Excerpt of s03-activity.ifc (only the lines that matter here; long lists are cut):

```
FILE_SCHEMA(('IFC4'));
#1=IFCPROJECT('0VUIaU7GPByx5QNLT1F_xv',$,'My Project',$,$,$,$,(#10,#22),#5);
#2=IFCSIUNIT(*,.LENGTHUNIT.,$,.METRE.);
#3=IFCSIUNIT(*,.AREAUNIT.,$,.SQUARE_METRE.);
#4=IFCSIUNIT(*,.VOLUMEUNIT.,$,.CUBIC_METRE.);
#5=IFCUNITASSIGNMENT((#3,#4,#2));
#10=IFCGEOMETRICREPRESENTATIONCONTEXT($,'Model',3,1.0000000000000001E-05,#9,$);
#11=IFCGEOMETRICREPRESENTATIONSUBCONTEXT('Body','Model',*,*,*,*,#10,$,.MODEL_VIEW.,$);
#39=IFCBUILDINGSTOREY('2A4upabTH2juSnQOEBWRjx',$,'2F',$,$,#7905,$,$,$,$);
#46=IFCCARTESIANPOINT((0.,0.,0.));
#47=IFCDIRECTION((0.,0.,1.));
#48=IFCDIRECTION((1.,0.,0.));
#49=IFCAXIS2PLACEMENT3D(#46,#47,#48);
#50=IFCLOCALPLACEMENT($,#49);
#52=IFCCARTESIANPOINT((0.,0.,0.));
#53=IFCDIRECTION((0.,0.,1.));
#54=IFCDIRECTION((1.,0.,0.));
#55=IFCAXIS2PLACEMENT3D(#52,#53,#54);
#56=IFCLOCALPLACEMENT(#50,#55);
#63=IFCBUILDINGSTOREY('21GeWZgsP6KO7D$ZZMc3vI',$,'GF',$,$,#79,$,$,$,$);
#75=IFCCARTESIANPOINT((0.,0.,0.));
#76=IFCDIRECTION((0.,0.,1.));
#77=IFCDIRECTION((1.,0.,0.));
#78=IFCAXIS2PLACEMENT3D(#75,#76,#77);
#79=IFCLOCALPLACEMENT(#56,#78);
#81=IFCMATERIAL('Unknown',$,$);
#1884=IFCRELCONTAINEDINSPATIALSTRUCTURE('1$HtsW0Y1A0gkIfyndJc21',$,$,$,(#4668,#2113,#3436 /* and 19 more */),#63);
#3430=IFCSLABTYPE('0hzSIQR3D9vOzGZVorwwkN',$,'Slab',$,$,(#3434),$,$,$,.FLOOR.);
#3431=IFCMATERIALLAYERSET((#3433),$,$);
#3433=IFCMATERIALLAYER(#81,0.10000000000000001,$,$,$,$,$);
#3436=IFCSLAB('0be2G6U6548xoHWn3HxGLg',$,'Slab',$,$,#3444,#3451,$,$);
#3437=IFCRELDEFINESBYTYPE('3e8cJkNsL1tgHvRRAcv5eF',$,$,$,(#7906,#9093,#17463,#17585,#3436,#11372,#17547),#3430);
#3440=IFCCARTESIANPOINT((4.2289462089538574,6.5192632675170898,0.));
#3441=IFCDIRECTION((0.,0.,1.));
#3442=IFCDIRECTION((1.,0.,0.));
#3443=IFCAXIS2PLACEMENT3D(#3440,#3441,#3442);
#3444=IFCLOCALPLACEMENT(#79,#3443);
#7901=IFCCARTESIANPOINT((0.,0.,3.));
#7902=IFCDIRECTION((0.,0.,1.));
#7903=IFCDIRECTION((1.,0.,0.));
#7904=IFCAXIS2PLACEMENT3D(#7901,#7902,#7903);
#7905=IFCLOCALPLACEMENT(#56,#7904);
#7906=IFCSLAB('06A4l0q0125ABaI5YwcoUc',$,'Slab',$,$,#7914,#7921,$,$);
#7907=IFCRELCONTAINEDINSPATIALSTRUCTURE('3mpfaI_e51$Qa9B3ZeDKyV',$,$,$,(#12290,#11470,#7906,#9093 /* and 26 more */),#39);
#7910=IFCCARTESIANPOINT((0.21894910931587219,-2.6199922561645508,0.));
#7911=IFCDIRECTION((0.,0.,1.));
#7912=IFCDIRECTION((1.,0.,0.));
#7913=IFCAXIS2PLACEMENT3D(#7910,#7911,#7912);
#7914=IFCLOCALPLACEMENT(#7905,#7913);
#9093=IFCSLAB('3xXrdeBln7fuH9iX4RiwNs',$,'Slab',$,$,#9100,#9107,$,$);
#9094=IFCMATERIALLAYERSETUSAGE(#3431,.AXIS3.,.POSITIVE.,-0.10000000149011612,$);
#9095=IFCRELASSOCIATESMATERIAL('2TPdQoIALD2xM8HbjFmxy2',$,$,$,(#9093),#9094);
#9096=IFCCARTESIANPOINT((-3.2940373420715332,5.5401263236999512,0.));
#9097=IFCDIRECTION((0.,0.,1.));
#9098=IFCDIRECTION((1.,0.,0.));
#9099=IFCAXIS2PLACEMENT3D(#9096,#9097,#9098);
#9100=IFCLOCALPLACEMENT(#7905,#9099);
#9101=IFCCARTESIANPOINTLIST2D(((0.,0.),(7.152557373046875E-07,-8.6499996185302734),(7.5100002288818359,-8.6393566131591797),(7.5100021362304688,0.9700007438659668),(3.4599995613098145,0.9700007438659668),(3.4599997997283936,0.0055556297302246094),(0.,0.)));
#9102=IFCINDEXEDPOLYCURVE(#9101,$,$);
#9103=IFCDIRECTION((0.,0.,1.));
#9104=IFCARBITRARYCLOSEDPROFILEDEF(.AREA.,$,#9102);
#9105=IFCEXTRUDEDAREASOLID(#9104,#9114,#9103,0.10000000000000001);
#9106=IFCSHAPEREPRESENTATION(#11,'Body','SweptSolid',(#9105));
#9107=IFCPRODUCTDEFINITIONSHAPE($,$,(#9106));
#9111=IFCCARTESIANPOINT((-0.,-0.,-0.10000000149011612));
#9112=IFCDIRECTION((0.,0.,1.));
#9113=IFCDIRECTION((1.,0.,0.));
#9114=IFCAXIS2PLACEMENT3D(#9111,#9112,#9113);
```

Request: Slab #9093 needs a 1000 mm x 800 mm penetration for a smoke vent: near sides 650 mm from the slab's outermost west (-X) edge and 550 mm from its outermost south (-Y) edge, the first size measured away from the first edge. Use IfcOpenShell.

```python
import numpy as np
import ifcopenshell
import ifcopenshell.api.feature
import ifcopenshell.api.geometry
import ifcopenshell.api.root
import ifcopenshell.geom
import ifcopenshell.util.placement
import ifcopenshell.util.representation
import ifcopenshell.util.shape
import ifcopenshell.util.unit

model = ifcopenshell.open("s03-activity.ifc")
unit_scale = ifcopenshell.util.unit.calculate_unit_scale(model)
settings = ifcopenshell.geom.settings()


def volume(element):
    """Net volume in cubic metres, openings subtracted."""
    shape = ifcopenshell.geom.create_shape(settings, element)
    return ifcopenshell.util.shape.get_volume(shape.geometry)


slab = model.by_guid("3xXrdeBln7fuH9iX4RiwNs")
before = volume(slab)

# Extent in the slab's own axes, in metres. The edges named are its -X and -Y sides.
slab_shape = ifcopenshell.geom.create_shape(settings, slab)
vertices = ifcopenshell.util.shape.get_vertices(slab_shape.geometry)
x_min, y_min, bottom = vertices.min(axis=0)
top = vertices[:, 2].max()

opening = ifcopenshell.api.root.create_entity(model, ifc_class="IfcOpeningElement", name="Smoke vent opening", predefined_type="OPENING")
context = ifcopenshell.util.representation.get_context(model, "Model", "Body", "MODEL_VIEW")
width, depth = 1, 0.8
outline = [(0.0, 0.0), (width, 0.0), (width, depth), (0.0, depth), (0.0, 0.0)]
# Overshoot both faces by 50 mm so the cut is clean.
shape = ifcopenshell.api.geometry.add_slab_representation(
    model, context=context, depth=top - bottom + 0.1, polyline=outline
)
ifcopenshell.api.geometry.assign_representation(model, product=opening, representation=shape)

matrix = ifcopenshell.util.placement.get_local_placement(slab.ObjectPlacement)
matrix[:, 3] = matrix @ np.append(np.array([x_min + 0.65, y_min + 0.55, bottom - 0.05]) / unit_scale, 1.0)
ifcopenshell.api.geometry.edit_object_placement(model, product=opening, matrix=matrix, is_si=False)
ifcopenshell.api.feature.add_feature(model, feature=opening, element=slab)

after = volume(slab)

print(f"slab volume {before:.3f} -> {after:.3f} m3")

model.write("s03-activity_v2.ifc")
```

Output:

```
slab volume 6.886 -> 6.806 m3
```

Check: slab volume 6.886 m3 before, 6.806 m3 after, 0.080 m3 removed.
